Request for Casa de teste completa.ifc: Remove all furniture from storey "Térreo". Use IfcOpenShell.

First a look at what the model holds.

```python
import ifcopenshell
import ifcopenshell.util.element

model = ifcopenshell.open("Casa de teste completa.ifc")
print(model.schema)
storey = next(s for s in model.by_type("IfcBuildingStorey") if s.Name == "Térreo")
furniture = [e for e in ifcopenshell.util.element.get_decomposition(storey) if e.is_a("IfcFurnishingElement")]
seen = {}
for e in furniture:
    element_type = ifcopenshell.util.element.get_type(e)
    name = element_type.Name if element_type not in (None, e) else None
    seen[name] = seen.get(name, 0) + 1
for name, count in sorted(seen.items(), key=str):
    print(count, "x", name)
```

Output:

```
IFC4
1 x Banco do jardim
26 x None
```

```python
import ifcopenshell
import ifcopenshell.api.root
import ifcopenshell.util.element

model = ifcopenshell.open("Casa de teste completa.ifc")

storey = next(s for s in model.by_type("IfcBuildingStorey") if s.Name == "Térreo")
furniture = [e for e in ifcopenshell.util.element.get_decomposition(storey) if e.is_a("IfcFurnishingElement")]

for e in furniture:
    ifcopenshell.api.root.remove_product(model, product=e)
print(len(furniture), "removed")

model.write("Casa de teste completa_updated.ifc")
```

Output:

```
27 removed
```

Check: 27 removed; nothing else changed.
